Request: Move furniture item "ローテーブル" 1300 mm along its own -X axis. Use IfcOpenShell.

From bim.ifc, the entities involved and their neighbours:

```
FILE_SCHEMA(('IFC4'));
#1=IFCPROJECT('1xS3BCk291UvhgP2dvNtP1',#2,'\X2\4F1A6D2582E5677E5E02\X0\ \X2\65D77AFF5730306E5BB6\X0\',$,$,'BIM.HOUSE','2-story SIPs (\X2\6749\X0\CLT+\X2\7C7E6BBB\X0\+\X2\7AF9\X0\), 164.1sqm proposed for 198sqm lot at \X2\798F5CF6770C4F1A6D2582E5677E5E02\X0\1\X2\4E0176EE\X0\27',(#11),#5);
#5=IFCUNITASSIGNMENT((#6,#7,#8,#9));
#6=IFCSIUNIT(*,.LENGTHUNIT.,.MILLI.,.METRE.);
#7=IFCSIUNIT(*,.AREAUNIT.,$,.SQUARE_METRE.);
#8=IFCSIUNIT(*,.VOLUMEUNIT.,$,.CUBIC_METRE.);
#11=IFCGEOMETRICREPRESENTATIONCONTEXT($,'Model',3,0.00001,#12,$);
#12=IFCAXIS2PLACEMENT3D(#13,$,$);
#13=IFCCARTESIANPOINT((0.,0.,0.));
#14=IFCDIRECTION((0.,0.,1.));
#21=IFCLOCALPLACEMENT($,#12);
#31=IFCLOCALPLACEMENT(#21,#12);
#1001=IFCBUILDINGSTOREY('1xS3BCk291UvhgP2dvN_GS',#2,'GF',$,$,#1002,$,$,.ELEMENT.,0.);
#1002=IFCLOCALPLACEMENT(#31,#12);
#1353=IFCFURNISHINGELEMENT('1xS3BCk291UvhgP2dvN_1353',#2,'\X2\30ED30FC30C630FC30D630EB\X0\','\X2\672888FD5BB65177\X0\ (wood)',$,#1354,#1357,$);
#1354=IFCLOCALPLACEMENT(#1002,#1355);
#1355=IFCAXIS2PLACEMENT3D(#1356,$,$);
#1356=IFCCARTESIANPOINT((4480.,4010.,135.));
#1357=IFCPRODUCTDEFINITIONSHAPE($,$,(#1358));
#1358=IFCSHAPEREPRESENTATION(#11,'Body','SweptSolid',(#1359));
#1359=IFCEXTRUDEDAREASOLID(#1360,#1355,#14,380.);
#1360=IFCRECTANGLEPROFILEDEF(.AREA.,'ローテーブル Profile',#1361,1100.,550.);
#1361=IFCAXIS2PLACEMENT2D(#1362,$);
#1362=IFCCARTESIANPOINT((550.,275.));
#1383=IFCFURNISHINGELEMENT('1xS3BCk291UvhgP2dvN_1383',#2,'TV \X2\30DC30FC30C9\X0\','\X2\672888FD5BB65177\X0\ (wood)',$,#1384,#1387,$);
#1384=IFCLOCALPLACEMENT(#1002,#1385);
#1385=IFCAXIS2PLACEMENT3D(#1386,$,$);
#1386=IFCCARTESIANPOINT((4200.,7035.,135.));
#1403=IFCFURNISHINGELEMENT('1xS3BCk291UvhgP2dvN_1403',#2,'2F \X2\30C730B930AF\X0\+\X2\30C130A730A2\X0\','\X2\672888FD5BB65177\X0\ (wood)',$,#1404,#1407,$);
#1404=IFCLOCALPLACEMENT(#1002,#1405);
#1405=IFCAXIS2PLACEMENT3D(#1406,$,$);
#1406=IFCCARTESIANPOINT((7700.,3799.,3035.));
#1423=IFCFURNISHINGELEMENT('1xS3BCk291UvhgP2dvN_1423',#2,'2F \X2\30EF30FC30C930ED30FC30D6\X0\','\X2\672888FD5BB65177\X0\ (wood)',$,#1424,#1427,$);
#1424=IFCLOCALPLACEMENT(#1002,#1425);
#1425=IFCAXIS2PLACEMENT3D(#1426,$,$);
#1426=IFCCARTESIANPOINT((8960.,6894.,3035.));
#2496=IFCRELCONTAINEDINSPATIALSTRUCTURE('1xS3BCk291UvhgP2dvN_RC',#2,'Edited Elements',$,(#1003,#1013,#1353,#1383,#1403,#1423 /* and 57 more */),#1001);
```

```python
import ifcopenshell
import ifcopenshell.api.geometry
import ifcopenshell.util.placement

model = ifcopenshell.open("bim.ifc")

item = model.by_id(1353)
matrix = ifcopenshell.util.placement.get_local_placement(item.ObjectPlacement)
matrix[:3, 3] -= matrix[:3, 0] * 1300.0
ifcopenshell.api.geometry.edit_object_placement(model, product=item, matrix=matrix, is_si=False)

print(ifcopenshell.util.placement.get_local_placement(item.ObjectPlacement).round(3) + 0.0)

model.write("bim_rev.ifc")
```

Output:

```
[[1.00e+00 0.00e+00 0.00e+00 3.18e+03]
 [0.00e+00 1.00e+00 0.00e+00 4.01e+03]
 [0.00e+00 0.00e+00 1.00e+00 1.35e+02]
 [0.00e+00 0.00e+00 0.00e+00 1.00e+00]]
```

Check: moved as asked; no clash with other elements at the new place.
